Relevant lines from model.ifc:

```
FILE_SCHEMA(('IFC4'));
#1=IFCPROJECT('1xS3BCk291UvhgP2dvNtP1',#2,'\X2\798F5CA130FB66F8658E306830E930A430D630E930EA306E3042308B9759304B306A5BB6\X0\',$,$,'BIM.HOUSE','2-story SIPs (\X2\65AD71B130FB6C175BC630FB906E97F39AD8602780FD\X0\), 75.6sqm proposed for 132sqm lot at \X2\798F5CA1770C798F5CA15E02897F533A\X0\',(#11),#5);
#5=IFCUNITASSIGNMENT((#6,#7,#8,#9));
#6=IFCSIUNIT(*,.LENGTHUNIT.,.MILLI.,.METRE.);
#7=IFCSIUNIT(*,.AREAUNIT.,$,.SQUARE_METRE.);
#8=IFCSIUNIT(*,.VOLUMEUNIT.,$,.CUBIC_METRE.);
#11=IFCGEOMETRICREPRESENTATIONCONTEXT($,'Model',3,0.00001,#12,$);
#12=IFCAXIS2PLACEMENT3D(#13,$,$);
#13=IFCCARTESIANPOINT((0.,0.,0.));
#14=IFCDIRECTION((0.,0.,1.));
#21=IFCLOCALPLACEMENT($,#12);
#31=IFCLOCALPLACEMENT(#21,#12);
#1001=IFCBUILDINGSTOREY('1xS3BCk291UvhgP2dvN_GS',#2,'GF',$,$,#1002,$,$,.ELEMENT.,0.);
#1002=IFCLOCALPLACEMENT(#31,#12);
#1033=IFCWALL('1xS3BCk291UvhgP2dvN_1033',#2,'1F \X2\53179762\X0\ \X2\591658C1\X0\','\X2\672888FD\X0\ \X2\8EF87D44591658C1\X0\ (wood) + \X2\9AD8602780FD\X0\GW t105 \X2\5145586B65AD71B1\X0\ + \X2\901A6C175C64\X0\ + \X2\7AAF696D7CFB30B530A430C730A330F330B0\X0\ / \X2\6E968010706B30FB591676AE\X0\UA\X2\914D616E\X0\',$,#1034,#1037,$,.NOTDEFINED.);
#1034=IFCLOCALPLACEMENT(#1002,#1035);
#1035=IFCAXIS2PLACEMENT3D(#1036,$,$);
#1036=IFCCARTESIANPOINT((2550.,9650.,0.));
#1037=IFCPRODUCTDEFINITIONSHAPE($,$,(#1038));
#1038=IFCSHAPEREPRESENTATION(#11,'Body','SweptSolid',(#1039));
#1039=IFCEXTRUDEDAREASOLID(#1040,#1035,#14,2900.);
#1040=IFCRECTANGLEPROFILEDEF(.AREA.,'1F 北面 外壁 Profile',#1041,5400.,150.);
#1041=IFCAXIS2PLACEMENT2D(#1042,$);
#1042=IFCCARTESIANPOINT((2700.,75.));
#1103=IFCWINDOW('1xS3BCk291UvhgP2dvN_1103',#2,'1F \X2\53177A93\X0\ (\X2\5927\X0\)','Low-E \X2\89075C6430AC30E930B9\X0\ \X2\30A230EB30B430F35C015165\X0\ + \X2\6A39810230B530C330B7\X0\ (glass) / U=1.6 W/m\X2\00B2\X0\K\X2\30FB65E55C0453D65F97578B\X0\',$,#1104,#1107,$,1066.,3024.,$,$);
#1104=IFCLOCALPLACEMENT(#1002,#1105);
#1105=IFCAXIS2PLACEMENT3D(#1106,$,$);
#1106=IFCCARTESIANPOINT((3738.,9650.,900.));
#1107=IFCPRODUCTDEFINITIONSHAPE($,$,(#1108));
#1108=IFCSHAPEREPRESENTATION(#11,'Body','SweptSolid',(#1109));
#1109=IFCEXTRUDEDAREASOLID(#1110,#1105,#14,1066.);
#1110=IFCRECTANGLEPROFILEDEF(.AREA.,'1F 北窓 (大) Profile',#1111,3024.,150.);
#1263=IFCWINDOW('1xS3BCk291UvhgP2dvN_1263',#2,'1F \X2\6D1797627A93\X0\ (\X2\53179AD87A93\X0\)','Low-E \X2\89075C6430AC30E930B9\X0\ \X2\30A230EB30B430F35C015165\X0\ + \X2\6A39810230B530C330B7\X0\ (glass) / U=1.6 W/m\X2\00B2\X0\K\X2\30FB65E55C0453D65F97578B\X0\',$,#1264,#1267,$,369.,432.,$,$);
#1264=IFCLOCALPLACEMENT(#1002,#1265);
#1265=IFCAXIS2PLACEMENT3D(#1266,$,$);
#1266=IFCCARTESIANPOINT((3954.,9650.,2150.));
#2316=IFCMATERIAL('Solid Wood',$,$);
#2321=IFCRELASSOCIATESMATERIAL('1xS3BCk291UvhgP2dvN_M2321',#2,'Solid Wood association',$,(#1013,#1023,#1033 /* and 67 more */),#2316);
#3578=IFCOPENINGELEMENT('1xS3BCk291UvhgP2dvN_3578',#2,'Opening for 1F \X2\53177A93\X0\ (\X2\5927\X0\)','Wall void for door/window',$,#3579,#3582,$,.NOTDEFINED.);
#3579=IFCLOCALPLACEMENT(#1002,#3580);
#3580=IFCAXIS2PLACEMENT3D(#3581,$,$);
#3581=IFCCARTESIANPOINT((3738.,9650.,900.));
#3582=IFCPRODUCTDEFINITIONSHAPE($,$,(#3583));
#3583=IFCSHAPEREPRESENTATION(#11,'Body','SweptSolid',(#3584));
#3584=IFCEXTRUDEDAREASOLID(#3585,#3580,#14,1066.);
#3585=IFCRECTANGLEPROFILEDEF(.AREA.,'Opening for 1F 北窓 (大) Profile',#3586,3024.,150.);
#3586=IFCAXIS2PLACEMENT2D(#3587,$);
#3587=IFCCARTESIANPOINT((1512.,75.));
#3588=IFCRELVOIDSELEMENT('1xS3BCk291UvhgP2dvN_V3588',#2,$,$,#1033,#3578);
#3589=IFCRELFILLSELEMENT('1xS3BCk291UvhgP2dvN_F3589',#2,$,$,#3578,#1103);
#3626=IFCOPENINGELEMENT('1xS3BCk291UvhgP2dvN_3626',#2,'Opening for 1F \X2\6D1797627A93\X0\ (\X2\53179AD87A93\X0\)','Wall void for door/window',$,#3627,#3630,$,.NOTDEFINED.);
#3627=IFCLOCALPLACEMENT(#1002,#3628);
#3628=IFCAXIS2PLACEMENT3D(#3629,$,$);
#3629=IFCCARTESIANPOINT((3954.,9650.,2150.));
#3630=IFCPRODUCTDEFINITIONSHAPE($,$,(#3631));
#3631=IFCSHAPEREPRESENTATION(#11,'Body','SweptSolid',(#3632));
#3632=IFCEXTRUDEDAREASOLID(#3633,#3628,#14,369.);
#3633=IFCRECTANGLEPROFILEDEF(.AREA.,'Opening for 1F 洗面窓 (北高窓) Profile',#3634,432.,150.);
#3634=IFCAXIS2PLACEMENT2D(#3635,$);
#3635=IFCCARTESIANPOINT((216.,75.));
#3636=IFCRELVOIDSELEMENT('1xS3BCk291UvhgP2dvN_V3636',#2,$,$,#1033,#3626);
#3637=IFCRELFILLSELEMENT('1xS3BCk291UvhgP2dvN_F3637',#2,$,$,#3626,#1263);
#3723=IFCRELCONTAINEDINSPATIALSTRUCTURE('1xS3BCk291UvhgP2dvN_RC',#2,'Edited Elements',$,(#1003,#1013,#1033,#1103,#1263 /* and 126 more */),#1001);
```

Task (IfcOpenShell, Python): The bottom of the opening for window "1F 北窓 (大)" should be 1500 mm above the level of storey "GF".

```python
import numpy as np
import ifcopenshell
import ifcopenshell.api.geometry
import ifcopenshell.geom
import ifcopenshell.util.element
import ifcopenshell.util.placement
import ifcopenshell.util.shape
import ifcopenshell.util.unit

model = ifcopenshell.open("model.ifc")
unit_scale = ifcopenshell.util.unit.calculate_unit_scale(model)

window = model.by_guid("1xS3BCk291UvhgP2dvN_1103")
opening = window.FillsVoids[0].RelatingOpeningElement
storey = ifcopenshell.util.element.get_container(window, ifc_class="IfcBuildingStorey")
level = ifcopenshell.util.placement.get_local_placement(storey.ObjectPlacement)[2, 3]

# The opening's origin need not be at the sill, so measure its lowest point.
shape = ifcopenshell.geom.create_shape(ifcopenshell.geom.settings(), opening)
bottom = ifcopenshell.util.shape.get_shape_bottom_elevation(shape, shape.geometry) / unit_scale
dz = level + 1.5 / unit_scale - bottom

shift = np.array([0.0, 0.0, dz])
# The window is not placed relative to its opening, so move both.
for product in (opening, window):
    matrix = ifcopenshell.util.placement.get_local_placement(product.ObjectPlacement)
    matrix[:3, 3] += shift
    ifcopenshell.api.geometry.edit_object_placement(model, product=product, matrix=matrix, is_si=False)

print(f"moved by {dz * unit_scale:+.3f} m")

model.write("model_updated.ifc")
```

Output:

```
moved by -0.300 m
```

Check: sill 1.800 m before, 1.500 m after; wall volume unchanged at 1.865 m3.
